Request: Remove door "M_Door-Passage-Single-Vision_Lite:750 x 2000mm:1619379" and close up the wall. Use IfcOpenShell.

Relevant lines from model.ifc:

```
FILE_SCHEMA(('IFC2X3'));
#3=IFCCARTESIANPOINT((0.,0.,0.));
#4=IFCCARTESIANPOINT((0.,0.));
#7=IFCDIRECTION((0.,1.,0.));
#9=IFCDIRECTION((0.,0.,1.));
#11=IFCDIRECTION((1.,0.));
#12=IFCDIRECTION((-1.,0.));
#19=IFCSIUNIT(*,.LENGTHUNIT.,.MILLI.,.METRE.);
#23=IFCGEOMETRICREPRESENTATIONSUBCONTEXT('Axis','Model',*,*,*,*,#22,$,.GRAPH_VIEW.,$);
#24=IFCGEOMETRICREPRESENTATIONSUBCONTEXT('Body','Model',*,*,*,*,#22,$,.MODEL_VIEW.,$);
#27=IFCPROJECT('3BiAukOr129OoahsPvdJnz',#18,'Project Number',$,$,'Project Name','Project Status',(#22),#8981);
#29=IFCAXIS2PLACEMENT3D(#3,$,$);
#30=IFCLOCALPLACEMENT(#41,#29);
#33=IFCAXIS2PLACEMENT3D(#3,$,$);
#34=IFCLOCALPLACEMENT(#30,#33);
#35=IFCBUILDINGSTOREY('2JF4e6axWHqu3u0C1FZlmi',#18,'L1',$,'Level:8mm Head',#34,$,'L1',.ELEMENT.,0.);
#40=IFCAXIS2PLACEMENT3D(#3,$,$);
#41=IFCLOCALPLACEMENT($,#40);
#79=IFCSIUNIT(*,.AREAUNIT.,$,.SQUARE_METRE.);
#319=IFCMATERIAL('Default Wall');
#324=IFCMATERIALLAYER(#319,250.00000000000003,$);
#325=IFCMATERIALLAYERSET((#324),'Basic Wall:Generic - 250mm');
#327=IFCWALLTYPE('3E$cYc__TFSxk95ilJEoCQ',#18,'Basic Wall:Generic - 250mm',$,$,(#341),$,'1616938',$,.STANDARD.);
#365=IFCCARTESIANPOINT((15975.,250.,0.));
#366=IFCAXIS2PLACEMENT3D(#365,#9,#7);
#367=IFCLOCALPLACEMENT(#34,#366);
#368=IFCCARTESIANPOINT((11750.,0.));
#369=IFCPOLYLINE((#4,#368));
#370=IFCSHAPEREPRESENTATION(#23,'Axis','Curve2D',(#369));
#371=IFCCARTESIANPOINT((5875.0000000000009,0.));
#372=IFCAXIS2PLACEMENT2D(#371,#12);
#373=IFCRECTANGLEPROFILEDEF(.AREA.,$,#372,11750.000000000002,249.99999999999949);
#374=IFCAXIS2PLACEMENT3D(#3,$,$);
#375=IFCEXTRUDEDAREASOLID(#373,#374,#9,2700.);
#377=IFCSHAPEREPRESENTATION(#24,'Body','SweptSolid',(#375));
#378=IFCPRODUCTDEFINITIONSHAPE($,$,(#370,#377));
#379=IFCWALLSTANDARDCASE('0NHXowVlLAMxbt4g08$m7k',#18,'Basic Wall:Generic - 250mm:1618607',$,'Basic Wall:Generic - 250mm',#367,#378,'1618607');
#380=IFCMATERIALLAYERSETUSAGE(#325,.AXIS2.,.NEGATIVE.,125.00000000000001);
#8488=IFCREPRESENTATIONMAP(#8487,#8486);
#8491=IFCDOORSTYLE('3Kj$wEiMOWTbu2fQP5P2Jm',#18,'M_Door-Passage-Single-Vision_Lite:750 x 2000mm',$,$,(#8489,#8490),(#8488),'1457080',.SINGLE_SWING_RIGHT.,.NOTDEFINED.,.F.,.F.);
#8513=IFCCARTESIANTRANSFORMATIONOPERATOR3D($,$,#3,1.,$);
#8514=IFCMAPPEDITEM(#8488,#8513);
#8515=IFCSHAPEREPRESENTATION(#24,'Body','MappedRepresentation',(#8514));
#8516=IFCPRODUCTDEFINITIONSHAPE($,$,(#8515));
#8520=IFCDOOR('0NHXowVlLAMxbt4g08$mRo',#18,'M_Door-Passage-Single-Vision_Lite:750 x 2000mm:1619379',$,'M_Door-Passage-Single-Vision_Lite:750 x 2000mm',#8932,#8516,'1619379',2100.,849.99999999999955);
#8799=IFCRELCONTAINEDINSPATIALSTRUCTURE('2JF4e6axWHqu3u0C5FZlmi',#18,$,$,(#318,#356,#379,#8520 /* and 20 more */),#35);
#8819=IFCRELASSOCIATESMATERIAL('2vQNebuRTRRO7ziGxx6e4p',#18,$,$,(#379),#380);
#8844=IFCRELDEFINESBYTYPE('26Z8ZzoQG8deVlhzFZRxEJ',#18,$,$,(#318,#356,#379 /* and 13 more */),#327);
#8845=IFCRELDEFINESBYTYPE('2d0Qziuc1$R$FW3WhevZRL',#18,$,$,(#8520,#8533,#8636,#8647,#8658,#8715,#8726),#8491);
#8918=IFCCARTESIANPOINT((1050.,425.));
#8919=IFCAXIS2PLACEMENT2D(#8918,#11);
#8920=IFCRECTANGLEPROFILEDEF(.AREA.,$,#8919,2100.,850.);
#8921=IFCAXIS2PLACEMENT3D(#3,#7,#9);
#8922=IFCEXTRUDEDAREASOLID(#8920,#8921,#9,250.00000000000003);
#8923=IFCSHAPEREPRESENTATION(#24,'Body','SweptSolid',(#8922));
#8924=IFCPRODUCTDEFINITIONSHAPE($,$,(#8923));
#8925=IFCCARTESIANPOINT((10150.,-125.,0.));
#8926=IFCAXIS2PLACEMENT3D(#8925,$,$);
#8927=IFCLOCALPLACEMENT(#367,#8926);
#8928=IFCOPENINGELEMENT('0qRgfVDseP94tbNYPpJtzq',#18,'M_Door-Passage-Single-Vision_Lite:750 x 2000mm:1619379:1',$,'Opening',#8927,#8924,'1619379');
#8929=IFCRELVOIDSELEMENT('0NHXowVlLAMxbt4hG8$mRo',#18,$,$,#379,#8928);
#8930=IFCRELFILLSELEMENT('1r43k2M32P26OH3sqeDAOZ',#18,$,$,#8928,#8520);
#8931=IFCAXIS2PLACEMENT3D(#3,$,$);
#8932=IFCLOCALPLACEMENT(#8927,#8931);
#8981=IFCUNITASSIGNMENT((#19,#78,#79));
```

```python
import ifcopenshell
import ifcopenshell.api.feature
import ifcopenshell.api.root
import ifcopenshell.geom
import ifcopenshell.util.shape

model = ifcopenshell.open("model.ifc")
settings = ifcopenshell.geom.settings()


def volume(element):
    """Net volume in cubic metres, openings subtracted."""
    shape = ifcopenshell.geom.create_shape(settings, element)
    return ifcopenshell.util.shape.get_volume(shape.geometry)


door = model.by_guid("0NHXowVlLAMxbt4g08$mRo")
opening = door.FillsVoids[0].RelatingOpeningElement
wall = opening.VoidsElements[0].RelatingBuildingElement
before = volume(wall)

ifcopenshell.api.root.remove_product(model, product=door)
ifcopenshell.api.feature.remove_feature(model, feature=opening)

after = volume(wall)

print(f"wall volume {before:.3f} -> {after:.3f} m3")

model.write("model-out.ifc")
```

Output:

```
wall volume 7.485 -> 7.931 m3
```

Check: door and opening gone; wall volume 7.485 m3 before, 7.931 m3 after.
